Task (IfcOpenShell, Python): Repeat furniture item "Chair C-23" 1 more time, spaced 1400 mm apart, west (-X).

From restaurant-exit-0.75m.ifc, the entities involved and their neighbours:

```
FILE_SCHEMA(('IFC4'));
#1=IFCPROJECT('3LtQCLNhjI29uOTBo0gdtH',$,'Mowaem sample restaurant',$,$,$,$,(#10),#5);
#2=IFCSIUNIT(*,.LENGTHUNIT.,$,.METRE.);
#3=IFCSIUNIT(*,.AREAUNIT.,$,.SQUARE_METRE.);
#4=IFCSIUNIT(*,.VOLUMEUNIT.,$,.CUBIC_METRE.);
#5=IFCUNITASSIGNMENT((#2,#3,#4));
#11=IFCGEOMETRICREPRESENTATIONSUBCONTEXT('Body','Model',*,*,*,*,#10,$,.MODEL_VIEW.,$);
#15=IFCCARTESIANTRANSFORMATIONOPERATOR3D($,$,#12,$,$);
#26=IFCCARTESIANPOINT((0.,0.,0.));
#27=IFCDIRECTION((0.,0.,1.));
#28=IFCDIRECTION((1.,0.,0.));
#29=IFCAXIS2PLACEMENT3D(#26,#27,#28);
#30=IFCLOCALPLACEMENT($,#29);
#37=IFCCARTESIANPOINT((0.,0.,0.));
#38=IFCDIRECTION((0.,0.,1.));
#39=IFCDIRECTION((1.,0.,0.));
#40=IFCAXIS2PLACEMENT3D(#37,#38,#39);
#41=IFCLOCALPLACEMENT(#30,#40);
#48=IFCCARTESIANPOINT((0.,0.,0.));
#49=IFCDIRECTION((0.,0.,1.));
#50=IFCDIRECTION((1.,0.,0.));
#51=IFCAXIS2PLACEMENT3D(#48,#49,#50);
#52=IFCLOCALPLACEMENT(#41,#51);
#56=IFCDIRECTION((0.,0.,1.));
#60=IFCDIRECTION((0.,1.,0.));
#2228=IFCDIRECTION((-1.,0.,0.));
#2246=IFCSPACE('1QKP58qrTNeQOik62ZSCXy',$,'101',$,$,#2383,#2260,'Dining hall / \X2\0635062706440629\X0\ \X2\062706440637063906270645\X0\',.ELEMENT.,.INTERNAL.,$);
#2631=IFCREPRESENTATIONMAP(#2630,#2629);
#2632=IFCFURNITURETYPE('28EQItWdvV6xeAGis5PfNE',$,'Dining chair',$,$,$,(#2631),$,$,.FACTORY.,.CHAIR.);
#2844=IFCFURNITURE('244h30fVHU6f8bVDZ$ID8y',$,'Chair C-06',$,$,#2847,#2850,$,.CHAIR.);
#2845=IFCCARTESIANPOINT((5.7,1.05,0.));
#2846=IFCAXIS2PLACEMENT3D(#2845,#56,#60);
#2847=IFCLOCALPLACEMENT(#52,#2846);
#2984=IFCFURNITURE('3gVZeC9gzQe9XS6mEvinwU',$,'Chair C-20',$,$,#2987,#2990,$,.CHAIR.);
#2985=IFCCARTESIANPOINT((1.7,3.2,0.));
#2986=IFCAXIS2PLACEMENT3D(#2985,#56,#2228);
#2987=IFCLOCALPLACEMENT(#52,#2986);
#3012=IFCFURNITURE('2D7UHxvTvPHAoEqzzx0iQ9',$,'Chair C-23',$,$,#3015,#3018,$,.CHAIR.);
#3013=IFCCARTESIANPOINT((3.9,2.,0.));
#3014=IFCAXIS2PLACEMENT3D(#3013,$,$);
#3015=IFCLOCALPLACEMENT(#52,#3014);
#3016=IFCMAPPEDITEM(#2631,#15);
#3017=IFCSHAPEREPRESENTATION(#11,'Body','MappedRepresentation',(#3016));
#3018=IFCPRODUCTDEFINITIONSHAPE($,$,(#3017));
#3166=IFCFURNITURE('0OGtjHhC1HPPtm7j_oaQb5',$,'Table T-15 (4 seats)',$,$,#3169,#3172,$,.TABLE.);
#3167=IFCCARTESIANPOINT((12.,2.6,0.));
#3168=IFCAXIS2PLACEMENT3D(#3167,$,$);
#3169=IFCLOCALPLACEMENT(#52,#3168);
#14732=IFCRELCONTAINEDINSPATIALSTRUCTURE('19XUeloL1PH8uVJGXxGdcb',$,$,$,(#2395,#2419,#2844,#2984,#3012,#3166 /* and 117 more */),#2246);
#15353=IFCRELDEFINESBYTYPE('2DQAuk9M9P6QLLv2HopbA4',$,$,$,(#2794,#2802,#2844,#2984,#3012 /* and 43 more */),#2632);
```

```python
import numpy as np
import ifcopenshell
import ifcopenshell.api.geometry
import ifcopenshell.api.root
import ifcopenshell.util.element
import ifcopenshell.util.placement
import ifcopenshell.util.unit

model = ifcopenshell.open("restaurant-exit-0.75m.ifc")
unit_scale = ifcopenshell.util.unit.calculate_unit_scale(model)

source = model.by_guid("2D7UHxvTvPHAoEqzzx0iQ9")
base = ifcopenshell.util.placement.get_local_placement(source.ObjectPlacement)
step = np.array([-1.0, 0.0, 0.0]) * 1.4 / unit_scale

for i in range(1, 2):
    copy = ifcopenshell.api.root.copy_class(model, product=source)
    copy.Representation = ifcopenshell.util.element.copy_deep(
        model, source.Representation, exclude=["IfcGeometricRepresentationContext", "IfcRepresentationMap"]
    )
    matrix = base.copy()
    matrix[:3, 3] += i * step
    print("added at", matrix[:3, 3].round(3) + 0.0)
    ifcopenshell.api.geometry.edit_object_placement(model, product=copy, matrix=matrix, is_si=False)

model.write("restaurant-exit-0.75m_v2.ifc")
```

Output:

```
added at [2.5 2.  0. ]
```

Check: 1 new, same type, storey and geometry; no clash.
